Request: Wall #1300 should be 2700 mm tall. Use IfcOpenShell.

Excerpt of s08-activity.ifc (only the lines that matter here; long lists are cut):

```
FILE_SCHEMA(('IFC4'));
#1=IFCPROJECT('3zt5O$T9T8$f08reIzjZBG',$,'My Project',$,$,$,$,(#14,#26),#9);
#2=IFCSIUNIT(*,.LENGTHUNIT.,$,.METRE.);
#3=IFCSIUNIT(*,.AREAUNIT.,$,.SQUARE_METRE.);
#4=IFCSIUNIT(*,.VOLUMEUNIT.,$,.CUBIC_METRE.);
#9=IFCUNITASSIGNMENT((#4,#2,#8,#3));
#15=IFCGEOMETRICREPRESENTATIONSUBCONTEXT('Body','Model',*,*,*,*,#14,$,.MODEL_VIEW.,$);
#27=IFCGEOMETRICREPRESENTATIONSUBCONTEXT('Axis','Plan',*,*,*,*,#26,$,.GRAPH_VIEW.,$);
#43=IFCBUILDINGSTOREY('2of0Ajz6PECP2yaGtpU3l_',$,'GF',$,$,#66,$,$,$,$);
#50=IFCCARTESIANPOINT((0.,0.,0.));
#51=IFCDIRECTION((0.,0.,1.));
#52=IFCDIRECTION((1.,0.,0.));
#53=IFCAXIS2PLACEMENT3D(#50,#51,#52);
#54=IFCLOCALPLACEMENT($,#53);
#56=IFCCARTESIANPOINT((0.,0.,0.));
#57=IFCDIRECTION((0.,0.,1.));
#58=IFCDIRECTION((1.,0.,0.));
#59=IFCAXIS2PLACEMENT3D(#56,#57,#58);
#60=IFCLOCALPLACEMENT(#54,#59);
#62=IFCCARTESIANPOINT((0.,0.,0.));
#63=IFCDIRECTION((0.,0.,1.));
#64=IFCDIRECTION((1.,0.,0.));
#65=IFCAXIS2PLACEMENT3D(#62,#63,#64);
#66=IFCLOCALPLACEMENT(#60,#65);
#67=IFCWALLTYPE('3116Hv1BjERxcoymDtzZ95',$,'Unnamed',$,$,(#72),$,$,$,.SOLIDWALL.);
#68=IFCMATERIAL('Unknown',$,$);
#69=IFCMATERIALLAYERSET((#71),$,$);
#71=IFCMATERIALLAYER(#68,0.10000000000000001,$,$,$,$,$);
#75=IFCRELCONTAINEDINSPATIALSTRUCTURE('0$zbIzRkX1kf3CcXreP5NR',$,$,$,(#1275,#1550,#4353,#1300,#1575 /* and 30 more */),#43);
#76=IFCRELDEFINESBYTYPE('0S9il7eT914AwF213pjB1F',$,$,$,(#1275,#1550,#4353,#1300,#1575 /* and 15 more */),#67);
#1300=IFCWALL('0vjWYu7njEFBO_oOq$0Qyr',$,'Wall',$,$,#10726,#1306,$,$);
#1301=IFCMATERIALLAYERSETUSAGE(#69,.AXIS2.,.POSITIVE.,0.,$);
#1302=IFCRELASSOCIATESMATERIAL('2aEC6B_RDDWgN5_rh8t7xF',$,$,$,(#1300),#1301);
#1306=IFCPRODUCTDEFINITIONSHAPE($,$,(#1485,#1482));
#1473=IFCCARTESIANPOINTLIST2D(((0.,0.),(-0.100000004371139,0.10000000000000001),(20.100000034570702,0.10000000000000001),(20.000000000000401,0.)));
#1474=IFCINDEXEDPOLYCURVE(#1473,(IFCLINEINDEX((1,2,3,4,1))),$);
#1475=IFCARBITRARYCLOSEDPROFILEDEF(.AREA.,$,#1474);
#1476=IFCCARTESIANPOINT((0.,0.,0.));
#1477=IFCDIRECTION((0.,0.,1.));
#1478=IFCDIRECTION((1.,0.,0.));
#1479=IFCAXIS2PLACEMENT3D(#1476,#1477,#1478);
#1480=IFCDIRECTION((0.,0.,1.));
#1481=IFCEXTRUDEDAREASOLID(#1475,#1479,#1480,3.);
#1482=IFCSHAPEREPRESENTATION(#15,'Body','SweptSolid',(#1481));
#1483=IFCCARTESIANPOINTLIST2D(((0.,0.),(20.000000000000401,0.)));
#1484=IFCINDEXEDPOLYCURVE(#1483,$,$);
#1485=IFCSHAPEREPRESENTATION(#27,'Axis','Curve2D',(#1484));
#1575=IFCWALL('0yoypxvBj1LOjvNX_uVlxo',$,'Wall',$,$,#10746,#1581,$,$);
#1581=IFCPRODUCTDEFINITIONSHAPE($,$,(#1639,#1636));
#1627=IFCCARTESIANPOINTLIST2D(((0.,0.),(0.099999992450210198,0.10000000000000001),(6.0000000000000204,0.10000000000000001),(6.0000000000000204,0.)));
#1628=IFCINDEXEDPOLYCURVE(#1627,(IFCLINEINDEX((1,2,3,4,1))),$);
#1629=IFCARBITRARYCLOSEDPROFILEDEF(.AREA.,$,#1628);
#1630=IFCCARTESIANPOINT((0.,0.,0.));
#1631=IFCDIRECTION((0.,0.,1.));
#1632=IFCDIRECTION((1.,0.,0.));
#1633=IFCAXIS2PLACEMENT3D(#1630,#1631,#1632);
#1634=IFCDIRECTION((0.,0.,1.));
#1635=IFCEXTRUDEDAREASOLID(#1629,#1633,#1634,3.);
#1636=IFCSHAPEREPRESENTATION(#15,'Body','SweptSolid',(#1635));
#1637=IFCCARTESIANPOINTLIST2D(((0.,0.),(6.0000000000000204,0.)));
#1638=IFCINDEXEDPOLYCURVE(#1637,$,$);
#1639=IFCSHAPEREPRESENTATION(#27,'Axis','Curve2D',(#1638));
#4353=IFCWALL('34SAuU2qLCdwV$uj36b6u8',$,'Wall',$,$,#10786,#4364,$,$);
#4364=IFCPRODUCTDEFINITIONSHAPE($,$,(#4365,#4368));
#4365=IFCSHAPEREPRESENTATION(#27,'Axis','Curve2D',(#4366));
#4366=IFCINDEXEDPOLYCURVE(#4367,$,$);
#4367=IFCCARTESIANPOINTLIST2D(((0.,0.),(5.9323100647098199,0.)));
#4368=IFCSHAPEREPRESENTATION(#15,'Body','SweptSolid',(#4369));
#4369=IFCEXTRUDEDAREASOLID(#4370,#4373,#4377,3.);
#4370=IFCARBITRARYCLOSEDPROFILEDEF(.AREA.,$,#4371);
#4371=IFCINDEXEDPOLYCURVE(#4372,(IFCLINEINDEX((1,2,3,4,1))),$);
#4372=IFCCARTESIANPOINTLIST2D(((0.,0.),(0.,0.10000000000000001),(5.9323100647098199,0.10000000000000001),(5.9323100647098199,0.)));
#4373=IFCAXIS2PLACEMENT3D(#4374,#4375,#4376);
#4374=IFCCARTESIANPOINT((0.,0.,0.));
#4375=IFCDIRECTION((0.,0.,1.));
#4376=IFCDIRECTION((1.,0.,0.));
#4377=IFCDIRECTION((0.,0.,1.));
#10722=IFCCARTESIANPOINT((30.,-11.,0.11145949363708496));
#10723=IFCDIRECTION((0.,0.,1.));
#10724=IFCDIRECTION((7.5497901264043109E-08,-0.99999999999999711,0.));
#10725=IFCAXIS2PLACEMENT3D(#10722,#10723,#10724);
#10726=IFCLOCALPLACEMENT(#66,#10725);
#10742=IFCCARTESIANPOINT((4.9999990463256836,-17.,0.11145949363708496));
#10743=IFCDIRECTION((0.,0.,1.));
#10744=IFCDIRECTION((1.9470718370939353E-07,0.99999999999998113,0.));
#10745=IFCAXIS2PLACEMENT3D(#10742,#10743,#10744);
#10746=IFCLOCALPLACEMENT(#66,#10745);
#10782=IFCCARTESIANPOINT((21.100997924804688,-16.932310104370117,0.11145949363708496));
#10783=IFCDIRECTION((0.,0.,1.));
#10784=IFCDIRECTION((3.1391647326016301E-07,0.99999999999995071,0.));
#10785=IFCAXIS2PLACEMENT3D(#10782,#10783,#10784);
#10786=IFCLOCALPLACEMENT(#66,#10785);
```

```python
import ifcopenshell
import ifcopenshell.geom
import ifcopenshell.util.representation
import ifcopenshell.util.shape

model = ifcopenshell.open("s08-activity.ifc")
settings = ifcopenshell.geom.settings()


def volume(element):
    """Net volume in cubic metres, openings subtracted."""
    shape = ifcopenshell.geom.create_shape(settings, element)
    return ifcopenshell.util.shape.get_volume(shape.geometry)


wall = model.by_id(1300)
before = volume(wall)

body = ifcopenshell.util.representation.get_representation(wall, "Model", "Body")
solid = body.Items[0]
old_height = solid.Depth
solid.Depth = 2.7
after = volume(wall)

print(f"height {old_height:g} -> {solid.Depth:g}, volume {before:.3f} -> {after:.3f} m3")

model.write("s08-activity_rev.ifc")
```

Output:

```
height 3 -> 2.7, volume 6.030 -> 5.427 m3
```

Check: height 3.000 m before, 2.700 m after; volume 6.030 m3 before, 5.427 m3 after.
